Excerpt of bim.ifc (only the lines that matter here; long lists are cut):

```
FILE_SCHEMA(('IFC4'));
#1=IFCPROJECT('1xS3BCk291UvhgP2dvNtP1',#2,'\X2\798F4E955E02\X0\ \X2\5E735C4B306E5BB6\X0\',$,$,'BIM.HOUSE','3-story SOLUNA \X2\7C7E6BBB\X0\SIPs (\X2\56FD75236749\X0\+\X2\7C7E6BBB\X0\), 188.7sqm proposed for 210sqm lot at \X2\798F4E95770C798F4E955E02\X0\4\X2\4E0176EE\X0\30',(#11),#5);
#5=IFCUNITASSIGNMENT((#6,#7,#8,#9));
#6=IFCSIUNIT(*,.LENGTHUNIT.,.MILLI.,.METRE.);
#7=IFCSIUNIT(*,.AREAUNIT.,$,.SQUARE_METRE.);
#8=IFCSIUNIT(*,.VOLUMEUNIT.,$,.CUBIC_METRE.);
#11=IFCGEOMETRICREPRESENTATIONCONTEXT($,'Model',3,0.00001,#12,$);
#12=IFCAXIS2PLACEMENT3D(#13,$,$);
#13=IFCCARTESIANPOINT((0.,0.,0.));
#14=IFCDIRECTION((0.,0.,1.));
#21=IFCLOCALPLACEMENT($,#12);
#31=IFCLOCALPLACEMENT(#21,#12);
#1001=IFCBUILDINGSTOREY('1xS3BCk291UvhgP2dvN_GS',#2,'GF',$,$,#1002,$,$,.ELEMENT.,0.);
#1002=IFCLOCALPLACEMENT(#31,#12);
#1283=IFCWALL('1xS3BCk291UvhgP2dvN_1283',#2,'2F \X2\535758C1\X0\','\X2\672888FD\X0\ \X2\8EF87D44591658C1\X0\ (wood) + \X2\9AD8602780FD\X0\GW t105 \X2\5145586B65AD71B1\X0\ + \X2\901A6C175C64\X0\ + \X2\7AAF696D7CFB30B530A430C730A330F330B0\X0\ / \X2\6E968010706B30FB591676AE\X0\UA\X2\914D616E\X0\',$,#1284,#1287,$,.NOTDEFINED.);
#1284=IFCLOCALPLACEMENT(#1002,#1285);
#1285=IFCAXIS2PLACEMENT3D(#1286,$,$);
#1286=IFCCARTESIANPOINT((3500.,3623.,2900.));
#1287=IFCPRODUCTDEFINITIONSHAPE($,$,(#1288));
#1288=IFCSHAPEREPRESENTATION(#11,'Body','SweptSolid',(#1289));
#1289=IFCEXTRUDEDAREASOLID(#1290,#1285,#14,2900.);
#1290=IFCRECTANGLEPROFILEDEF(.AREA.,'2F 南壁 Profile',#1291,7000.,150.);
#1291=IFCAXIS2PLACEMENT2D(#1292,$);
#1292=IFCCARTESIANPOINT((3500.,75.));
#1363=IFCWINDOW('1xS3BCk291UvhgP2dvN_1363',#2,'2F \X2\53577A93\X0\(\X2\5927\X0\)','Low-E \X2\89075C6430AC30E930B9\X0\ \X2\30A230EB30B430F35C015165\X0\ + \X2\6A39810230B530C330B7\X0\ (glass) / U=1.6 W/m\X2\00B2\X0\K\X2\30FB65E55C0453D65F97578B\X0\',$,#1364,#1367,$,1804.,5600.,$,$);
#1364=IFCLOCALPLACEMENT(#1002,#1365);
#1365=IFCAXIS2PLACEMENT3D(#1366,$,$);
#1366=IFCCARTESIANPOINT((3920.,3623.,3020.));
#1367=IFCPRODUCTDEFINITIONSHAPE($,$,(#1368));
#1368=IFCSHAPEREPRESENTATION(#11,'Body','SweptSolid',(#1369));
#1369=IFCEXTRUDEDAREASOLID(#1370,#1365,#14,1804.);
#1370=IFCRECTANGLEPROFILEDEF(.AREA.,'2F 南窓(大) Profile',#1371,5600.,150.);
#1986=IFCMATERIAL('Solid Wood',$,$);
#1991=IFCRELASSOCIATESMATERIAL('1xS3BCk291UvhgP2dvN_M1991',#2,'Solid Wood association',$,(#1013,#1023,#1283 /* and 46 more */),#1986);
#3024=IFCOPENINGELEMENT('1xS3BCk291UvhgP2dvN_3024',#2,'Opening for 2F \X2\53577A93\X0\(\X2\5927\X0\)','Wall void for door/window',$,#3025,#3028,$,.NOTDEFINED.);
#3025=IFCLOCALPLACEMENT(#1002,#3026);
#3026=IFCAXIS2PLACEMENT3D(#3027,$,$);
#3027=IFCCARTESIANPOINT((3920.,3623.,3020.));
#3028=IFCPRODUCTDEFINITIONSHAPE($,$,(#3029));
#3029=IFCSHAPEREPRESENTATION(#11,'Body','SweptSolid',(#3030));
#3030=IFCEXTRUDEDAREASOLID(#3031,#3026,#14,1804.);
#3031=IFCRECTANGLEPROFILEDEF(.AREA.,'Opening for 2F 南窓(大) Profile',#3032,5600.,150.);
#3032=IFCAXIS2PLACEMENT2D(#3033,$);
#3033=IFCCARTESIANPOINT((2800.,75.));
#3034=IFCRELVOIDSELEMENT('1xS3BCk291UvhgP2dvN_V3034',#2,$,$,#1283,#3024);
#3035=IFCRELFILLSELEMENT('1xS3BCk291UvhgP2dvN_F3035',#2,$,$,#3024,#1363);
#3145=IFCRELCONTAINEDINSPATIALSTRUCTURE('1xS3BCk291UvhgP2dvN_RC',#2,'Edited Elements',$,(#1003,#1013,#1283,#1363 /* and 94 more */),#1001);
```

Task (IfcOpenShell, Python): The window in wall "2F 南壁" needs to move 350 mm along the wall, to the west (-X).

```python
import ifcopenshell
import ifcopenshell.api.geometry
import ifcopenshell.util.placement
import ifcopenshell.util.unit

model = ifcopenshell.open("bim.ifc")
unit_scale = ifcopenshell.util.unit.calculate_unit_scale(model)

window = model.by_guid("1xS3BCk291UvhgP2dvN_1363")
opening = window.FillsVoids[0].RelatingOpeningElement
wall = opening.VoidsElements[0].RelatingBuildingElement

wall_matrix = ifcopenshell.util.placement.get_local_placement(wall.ObjectPlacement)
shift = wall_matrix[:3, 0] * -0.35 / unit_scale
before = ifcopenshell.util.placement.get_local_placement(window.ObjectPlacement)[:3, 3].copy()

# The window is not placed relative to its opening, so move both.
for product in (opening, window):
    matrix = ifcopenshell.util.placement.get_local_placement(product.ObjectPlacement)
    matrix[:3, 3] += shift
    ifcopenshell.api.geometry.edit_object_placement(model, product=product, matrix=matrix, is_si=False)

after = ifcopenshell.util.placement.get_local_placement(window.ObjectPlacement)[:3, 3]
print("window moved by", (after - before).round(3) + 0.0)

model.write("bim_v2.ifc")
```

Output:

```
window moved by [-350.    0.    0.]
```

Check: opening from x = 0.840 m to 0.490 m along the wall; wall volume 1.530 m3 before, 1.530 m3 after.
